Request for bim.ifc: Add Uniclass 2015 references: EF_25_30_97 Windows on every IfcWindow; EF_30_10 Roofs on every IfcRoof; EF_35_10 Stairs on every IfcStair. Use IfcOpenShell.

First a look at what the model holds.

```python
import ifcopenshell

model = ifcopenshell.open("bim.ifc")
print(model.schema)
print("classifications:", [c.Name for c in model.by_type("IfcClassification")])
for ifc_class in ("IfcDoor", "IfcRoof", "IfcStair", "IfcWall", "IfcWindow"):
    print(ifc_class, len(model.by_type(ifc_class)))
```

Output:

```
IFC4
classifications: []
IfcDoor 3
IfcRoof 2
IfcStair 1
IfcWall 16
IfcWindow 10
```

```python
import ifcopenshell
import ifcopenshell.api.classification

model = ifcopenshell.open("bim.ifc")

system = ifcopenshell.api.classification.add_classification(model, classification="Uniclass 2015")

codes = {
    "IfcWindow": ("EF_25_30_97", "Windows"),
    "IfcRoof": ("EF_30_10", "Roofs"),
    "IfcStair": ("EF_35_10", "Stairs"),
}
for ifc_class, (code, name) in codes.items():
    products = model.by_type(ifc_class)
    ifcopenshell.api.classification.add_reference(
        model, products=products, classification=system, identification=code, name=name
    )
    print(code, len(products))

model.write("bim_rev.ifc")
```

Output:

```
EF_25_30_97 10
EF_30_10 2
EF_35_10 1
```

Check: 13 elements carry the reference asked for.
